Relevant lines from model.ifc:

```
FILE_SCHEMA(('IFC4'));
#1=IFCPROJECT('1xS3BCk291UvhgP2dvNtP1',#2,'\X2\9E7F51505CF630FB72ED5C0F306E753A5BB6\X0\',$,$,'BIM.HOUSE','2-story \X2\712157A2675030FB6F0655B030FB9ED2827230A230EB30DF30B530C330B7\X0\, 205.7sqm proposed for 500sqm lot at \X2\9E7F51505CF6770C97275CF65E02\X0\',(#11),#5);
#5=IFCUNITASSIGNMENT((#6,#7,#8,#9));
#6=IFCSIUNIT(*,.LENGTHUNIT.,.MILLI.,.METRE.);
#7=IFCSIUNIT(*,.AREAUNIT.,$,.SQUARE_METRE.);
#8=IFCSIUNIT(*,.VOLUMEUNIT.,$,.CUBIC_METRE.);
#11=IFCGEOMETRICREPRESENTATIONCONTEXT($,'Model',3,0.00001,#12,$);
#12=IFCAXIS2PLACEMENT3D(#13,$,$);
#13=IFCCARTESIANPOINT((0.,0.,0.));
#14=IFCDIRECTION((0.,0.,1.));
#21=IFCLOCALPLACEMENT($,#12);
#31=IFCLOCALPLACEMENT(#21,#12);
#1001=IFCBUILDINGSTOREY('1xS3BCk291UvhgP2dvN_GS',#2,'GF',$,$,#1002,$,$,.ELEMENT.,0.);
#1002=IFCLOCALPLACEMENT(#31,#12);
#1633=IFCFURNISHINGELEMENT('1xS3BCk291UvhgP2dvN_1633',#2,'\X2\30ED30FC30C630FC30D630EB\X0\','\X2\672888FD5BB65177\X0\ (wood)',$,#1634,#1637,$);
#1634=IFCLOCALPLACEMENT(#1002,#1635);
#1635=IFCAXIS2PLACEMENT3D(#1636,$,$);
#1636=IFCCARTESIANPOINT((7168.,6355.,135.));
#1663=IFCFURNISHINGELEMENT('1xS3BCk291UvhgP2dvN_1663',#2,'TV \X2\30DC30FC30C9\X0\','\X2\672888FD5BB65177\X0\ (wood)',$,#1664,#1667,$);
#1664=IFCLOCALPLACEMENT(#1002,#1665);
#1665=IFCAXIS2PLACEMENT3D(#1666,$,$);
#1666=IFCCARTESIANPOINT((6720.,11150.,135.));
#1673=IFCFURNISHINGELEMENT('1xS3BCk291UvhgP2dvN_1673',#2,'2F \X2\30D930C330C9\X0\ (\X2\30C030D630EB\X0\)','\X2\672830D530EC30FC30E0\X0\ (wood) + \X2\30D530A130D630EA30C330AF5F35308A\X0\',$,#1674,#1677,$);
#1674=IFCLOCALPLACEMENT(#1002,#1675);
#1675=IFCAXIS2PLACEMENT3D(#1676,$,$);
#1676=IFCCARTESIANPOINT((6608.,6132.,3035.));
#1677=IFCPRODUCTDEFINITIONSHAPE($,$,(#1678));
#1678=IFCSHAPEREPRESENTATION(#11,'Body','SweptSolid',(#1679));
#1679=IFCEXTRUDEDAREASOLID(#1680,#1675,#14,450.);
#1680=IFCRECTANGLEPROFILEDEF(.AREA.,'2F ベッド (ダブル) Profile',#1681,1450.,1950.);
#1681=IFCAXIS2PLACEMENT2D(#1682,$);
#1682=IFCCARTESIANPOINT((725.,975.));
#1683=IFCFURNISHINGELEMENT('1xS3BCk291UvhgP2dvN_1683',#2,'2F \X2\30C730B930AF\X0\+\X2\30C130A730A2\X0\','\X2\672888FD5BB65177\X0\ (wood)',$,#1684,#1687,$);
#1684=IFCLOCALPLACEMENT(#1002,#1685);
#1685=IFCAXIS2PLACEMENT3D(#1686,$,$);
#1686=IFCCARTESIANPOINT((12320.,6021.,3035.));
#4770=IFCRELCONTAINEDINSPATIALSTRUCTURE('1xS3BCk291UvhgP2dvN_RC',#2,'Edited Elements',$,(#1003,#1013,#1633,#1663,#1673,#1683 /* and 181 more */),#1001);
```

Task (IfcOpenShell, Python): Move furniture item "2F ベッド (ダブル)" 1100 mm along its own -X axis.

```python
import ifcopenshell
import ifcopenshell.api.geometry
import ifcopenshell.util.placement
import ifcopenshell.util.unit

model = ifcopenshell.open("model.ifc")
unit_scale = ifcopenshell.util.unit.calculate_unit_scale(model)

item = model.by_id(1673)
matrix = ifcopenshell.util.placement.get_local_placement(item.ObjectPlacement)
matrix[:3, 3] -= matrix[:3, 0] * 1.1 / unit_scale
ifcopenshell.api.geometry.edit_object_placement(model, product=item, matrix=matrix, is_si=False)

print(ifcopenshell.util.placement.get_local_placement(item.ObjectPlacement).round(3) + 0.0)

model.write("model_edited.ifc")
```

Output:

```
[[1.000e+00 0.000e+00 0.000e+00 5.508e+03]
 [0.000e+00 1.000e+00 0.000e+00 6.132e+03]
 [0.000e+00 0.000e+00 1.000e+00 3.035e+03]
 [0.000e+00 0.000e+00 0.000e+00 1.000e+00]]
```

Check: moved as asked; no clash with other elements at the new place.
